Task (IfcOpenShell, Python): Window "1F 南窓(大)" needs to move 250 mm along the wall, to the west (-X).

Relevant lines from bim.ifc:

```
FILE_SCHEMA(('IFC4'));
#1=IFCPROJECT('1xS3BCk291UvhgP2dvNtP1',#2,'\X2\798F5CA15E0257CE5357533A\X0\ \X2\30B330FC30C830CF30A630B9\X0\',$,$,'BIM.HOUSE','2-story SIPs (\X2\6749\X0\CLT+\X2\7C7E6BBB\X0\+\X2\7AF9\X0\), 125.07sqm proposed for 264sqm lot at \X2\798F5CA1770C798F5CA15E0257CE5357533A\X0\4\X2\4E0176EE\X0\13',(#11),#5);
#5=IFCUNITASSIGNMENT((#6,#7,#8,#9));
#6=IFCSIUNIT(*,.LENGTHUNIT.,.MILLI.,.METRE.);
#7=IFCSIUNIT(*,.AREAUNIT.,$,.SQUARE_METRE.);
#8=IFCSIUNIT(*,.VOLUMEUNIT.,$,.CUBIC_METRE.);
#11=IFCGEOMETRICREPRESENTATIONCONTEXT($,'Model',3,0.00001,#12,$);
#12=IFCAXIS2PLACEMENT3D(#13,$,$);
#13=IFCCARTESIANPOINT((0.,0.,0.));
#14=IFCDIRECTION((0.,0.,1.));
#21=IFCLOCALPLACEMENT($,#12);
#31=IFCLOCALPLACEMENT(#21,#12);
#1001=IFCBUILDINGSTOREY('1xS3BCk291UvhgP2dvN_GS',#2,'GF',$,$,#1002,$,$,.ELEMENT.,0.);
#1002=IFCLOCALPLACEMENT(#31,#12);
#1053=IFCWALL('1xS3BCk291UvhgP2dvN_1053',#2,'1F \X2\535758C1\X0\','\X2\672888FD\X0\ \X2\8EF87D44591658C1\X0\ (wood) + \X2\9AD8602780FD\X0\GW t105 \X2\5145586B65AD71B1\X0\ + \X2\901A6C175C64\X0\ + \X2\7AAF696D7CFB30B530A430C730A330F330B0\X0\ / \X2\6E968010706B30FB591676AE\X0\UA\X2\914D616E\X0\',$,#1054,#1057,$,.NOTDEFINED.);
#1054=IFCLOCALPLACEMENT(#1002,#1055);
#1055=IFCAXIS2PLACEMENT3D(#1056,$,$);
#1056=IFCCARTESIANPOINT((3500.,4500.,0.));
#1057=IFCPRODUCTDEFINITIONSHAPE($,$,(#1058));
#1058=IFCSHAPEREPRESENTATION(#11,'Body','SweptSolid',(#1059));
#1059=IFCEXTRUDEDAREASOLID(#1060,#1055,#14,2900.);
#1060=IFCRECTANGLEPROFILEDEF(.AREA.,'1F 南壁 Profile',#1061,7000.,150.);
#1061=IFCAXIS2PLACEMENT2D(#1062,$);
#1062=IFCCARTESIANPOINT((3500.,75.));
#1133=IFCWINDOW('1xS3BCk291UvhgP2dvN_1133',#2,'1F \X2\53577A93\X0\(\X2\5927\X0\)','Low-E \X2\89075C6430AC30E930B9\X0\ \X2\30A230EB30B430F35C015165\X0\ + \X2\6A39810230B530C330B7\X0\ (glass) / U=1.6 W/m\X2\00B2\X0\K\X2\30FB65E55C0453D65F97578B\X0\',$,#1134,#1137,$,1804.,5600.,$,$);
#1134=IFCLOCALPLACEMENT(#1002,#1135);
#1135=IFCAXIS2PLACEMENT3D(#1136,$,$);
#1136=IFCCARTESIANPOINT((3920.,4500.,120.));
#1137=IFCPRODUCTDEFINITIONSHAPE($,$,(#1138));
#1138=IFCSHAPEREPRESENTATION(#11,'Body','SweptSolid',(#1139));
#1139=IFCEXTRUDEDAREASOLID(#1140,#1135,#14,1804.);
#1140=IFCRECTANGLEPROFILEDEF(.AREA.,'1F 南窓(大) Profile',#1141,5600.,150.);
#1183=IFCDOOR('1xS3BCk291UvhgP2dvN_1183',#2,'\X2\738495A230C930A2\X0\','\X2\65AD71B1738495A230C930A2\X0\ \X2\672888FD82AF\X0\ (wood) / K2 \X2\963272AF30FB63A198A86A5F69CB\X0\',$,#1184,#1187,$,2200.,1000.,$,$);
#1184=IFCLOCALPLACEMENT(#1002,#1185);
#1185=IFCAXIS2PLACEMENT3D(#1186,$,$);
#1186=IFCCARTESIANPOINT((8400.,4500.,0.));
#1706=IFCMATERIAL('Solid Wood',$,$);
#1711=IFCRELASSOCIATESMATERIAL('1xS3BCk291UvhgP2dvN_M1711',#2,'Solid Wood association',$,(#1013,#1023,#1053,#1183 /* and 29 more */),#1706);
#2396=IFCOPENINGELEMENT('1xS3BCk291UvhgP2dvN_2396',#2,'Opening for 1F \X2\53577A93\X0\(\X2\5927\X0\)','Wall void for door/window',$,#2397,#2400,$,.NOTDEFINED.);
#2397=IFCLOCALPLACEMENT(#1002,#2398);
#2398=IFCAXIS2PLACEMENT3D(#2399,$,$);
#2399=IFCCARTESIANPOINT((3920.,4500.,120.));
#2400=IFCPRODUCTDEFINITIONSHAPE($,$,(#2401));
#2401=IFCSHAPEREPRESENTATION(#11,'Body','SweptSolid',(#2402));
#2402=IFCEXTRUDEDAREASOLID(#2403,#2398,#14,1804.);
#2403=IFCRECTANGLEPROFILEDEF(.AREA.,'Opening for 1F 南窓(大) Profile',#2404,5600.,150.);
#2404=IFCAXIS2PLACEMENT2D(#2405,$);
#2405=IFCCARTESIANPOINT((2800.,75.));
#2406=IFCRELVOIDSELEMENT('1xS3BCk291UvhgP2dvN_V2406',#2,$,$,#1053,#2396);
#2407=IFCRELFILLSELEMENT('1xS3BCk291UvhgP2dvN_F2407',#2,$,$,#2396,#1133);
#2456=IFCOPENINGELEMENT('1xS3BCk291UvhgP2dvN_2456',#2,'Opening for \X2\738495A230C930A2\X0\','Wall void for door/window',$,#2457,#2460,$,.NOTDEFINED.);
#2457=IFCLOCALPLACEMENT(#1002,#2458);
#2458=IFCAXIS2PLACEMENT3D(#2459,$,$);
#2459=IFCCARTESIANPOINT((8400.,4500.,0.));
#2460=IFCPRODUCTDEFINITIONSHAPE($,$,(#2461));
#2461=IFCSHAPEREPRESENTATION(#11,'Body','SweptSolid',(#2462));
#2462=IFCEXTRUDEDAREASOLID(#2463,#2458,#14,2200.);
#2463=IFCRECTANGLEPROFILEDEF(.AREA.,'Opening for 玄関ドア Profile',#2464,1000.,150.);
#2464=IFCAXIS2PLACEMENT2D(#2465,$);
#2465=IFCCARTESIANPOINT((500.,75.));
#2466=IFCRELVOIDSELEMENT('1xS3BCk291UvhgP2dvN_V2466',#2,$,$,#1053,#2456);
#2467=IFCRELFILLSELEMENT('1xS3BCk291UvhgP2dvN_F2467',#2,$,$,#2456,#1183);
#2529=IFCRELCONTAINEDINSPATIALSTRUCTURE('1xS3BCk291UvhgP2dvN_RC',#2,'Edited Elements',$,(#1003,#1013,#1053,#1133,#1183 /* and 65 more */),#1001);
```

```python
import ifcopenshell
import ifcopenshell.api.geometry
import ifcopenshell.util.placement

model = ifcopenshell.open("bim.ifc")

window = model.by_guid("1xS3BCk291UvhgP2dvN_1133")
opening = window.FillsVoids[0].RelatingOpeningElement
wall = opening.VoidsElements[0].RelatingBuildingElement

wall_matrix = ifcopenshell.util.placement.get_local_placement(wall.ObjectPlacement)
shift = wall_matrix[:3, 0] * -250.0
before = ifcopenshell.util.placement.get_local_placement(window.ObjectPlacement)[:3, 3].copy()

# The window is not placed relative to its opening, so move both.
for product in (opening, window):
    matrix = ifcopenshell.util.placement.get_local_placement(product.ObjectPlacement)
    matrix[:3, 3] += shift
    ifcopenshell.api.geometry.edit_object_placement(model, product=product, matrix=matrix, is_si=False)

after = ifcopenshell.util.placement.get_local_placement(window.ObjectPlacement)[:3, 3]
print("window moved by", (after - before).round(3) + 0.0)

model.write("bim_v2.ifc")
```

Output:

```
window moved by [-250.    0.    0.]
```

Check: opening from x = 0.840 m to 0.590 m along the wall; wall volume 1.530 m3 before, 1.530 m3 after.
